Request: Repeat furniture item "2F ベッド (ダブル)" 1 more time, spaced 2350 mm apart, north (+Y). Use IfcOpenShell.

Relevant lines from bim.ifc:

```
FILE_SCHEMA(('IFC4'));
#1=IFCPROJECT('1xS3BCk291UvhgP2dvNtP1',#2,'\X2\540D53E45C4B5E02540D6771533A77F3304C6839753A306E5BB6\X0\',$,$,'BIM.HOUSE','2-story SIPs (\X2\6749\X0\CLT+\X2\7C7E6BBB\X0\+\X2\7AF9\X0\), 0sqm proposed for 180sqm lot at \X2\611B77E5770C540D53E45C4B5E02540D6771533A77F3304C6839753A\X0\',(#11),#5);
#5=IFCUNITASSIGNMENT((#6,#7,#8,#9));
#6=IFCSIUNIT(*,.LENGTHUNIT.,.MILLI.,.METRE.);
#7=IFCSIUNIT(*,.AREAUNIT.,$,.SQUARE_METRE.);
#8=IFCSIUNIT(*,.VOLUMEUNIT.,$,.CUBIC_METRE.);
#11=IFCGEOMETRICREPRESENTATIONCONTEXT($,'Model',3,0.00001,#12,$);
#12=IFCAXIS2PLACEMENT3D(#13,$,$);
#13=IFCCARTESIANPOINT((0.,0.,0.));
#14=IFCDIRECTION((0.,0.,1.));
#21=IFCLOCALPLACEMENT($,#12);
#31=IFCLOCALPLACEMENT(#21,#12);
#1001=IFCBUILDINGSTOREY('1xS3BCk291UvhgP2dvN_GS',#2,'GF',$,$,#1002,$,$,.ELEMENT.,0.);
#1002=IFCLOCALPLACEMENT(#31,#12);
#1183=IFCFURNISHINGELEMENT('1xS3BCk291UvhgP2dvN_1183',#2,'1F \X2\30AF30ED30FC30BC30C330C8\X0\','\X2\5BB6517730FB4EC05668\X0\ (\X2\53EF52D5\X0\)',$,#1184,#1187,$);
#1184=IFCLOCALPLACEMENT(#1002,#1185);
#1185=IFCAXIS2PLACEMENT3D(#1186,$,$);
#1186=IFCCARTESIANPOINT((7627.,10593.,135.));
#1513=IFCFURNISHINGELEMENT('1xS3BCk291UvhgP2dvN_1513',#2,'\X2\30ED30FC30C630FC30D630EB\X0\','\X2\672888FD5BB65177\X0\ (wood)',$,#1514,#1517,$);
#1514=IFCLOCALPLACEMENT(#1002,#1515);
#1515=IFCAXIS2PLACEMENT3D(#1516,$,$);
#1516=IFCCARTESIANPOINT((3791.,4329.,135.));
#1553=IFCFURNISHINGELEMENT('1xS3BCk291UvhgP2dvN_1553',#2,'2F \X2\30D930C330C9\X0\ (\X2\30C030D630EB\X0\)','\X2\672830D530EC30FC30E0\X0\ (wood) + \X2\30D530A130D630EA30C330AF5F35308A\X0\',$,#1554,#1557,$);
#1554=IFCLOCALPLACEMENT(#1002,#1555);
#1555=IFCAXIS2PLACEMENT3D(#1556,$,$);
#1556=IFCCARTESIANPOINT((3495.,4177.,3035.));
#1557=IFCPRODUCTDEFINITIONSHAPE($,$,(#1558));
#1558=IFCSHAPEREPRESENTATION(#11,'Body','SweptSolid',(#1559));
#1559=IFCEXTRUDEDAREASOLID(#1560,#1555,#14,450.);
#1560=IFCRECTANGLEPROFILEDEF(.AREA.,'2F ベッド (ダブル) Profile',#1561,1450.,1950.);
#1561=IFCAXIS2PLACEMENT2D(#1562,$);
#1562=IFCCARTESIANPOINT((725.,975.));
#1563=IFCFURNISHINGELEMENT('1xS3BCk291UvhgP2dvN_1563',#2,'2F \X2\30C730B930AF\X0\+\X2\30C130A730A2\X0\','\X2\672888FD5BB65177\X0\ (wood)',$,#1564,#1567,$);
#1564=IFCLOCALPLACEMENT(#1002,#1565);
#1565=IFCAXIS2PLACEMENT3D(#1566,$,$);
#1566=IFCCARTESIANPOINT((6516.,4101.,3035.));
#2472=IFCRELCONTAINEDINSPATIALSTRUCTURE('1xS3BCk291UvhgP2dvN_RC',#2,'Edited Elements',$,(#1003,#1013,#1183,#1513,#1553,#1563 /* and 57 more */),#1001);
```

```python
import numpy as np
import ifcopenshell
import ifcopenshell.api.geometry
import ifcopenshell.api.root
import ifcopenshell.util.element
import ifcopenshell.util.placement
import ifcopenshell.util.unit

model = ifcopenshell.open("bim.ifc")
unit_scale = ifcopenshell.util.unit.calculate_unit_scale(model)


def reuse_history(source, copy):
    """copy_class also copies each property set's owner history, people and application; keep the originals."""
    for rel in copy.IsDefinedBy:
        if rel.is_a("IfcRelDefinesByProperties") and (history := rel.RelatingPropertyDefinition.OwnerHistory):
            rel.RelatingPropertyDefinition.OwnerHistory = source.OwnerHistory
            ifcopenshell.util.element.remove_deep2(model, history)


source = model.by_guid("1xS3BCk291UvhgP2dvN_1553")
base = ifcopenshell.util.placement.get_local_placement(source.ObjectPlacement)
step = np.array([0.0, 1.0, 0.0]) * 2.35 / unit_scale

for i in range(1, 2):
    copy = ifcopenshell.api.root.copy_class(model, product=source)
    copy.Representation = ifcopenshell.util.element.copy_deep(
        model, source.Representation, exclude=["IfcGeometricRepresentationContext", "IfcRepresentationMap"]
    )
    reuse_history(source, copy)
    matrix = base.copy()
    matrix[:3, 3] += i * step
    print("added at", matrix[:3, 3].round(3) + 0.0)
    ifcopenshell.api.geometry.edit_object_placement(model, product=copy, matrix=matrix, is_si=False)

model.write("bim-out.ifc")
```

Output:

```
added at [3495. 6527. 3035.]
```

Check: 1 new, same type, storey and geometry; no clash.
